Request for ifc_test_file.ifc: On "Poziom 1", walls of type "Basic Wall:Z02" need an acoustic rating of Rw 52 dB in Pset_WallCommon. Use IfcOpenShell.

First a look at what the model holds.

```python
import ifcopenshell
import ifcopenshell.util.element

model = ifcopenshell.open("ifc_test_file.ifc")
print(model.schema)
storey = next(s for s in model.by_type("IfcBuildingStorey") if s.Name == "Poziom 1")
walls = [e for e in ifcopenshell.util.element.get_decomposition(storey) if e.is_a("IfcWall")]
seen = {}
for e in walls:
    element_type = ifcopenshell.util.element.get_type(e)
    key = (element_type.Name if element_type != e and element_type else None, ifcopenshell.util.element.get_pset(e, "Pset_WallCommon", "AcousticRating"))
    seen[key] = seen.get(key, 0) + 1
for (name, value), count in sorted(seen.items(), key=str):
    print(count, "x", name, "|", value)
```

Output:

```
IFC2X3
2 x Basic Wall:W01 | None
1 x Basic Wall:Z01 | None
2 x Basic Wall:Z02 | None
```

```python
import ifcopenshell
import ifcopenshell.api.pset
import ifcopenshell.util.element

model = ifcopenshell.open("ifc_test_file.ifc")

storey = next(s for s in model.by_type("IfcBuildingStorey") if s.Name == "Poziom 1")
walls = [e for e in ifcopenshell.util.element.get_decomposition(storey) if e.is_a("IfcWall")]

count = 0
for e in walls:
    element_type = ifcopenshell.util.element.get_type(e)
    if element_type in (None, e) or element_type.Name != "Basic Wall:Z02":
        continue
    # add_pset returns the element's existing set when there is one.
    pset = ifcopenshell.api.pset.add_pset(model, product=e, name="Pset_WallCommon")
    ifcopenshell.api.pset.edit_pset(model, pset=pset, properties={"AcousticRating": "Rw 52 dB"})
    count += 1

print(count, "walls updated")

model.write("ifc_test_file_edited.ifc")
```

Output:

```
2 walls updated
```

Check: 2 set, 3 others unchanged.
